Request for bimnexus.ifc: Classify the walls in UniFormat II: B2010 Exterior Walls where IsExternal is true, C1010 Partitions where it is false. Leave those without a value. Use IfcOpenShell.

First a look at what the model holds.

```python
import ifcopenshell
import ifcopenshell.util.element

model = ifcopenshell.open("bimnexus.ifc")
print(model.schema)
print("classifications:", [c.Name for c in model.by_type("IfcClassification")])
values = [ifcopenshell.util.element.get_pset(e, "Pset_WallCommon", "IsExternal") for e in model.by_type("IfcWall")]
for value in (True, False, None):
    print("IsExternal", value, values.count(value))
```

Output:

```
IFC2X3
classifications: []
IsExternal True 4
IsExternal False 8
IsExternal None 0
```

```python
import ifcopenshell
import ifcopenshell.api.classification
import ifcopenshell.util.element

model = ifcopenshell.open("bimnexus.ifc")

# IFC2X3 requires Source and Edition and has no link from the project to the system.
system = model.create_entity("IfcClassification", Source="ASTM", Edition="E1557", Name="UniFormat II")

walls = model.by_type("IfcWall")
external = {e: ifcopenshell.util.element.get_pset(e, "Pset_WallCommon", "IsExternal") for e in walls}
for flag, code, name in ((True, "B2010", "Exterior Walls"), (False, "C1010", "Partitions")):
    products = [e for e in walls if external[e] is flag]
    ifcopenshell.api.classification.add_reference(
        model, products=products, classification=system, identification=code, name=name
    )
    print(code, len(products))

model.write("bimnexus_updated.ifc")
```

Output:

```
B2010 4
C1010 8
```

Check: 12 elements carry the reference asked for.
